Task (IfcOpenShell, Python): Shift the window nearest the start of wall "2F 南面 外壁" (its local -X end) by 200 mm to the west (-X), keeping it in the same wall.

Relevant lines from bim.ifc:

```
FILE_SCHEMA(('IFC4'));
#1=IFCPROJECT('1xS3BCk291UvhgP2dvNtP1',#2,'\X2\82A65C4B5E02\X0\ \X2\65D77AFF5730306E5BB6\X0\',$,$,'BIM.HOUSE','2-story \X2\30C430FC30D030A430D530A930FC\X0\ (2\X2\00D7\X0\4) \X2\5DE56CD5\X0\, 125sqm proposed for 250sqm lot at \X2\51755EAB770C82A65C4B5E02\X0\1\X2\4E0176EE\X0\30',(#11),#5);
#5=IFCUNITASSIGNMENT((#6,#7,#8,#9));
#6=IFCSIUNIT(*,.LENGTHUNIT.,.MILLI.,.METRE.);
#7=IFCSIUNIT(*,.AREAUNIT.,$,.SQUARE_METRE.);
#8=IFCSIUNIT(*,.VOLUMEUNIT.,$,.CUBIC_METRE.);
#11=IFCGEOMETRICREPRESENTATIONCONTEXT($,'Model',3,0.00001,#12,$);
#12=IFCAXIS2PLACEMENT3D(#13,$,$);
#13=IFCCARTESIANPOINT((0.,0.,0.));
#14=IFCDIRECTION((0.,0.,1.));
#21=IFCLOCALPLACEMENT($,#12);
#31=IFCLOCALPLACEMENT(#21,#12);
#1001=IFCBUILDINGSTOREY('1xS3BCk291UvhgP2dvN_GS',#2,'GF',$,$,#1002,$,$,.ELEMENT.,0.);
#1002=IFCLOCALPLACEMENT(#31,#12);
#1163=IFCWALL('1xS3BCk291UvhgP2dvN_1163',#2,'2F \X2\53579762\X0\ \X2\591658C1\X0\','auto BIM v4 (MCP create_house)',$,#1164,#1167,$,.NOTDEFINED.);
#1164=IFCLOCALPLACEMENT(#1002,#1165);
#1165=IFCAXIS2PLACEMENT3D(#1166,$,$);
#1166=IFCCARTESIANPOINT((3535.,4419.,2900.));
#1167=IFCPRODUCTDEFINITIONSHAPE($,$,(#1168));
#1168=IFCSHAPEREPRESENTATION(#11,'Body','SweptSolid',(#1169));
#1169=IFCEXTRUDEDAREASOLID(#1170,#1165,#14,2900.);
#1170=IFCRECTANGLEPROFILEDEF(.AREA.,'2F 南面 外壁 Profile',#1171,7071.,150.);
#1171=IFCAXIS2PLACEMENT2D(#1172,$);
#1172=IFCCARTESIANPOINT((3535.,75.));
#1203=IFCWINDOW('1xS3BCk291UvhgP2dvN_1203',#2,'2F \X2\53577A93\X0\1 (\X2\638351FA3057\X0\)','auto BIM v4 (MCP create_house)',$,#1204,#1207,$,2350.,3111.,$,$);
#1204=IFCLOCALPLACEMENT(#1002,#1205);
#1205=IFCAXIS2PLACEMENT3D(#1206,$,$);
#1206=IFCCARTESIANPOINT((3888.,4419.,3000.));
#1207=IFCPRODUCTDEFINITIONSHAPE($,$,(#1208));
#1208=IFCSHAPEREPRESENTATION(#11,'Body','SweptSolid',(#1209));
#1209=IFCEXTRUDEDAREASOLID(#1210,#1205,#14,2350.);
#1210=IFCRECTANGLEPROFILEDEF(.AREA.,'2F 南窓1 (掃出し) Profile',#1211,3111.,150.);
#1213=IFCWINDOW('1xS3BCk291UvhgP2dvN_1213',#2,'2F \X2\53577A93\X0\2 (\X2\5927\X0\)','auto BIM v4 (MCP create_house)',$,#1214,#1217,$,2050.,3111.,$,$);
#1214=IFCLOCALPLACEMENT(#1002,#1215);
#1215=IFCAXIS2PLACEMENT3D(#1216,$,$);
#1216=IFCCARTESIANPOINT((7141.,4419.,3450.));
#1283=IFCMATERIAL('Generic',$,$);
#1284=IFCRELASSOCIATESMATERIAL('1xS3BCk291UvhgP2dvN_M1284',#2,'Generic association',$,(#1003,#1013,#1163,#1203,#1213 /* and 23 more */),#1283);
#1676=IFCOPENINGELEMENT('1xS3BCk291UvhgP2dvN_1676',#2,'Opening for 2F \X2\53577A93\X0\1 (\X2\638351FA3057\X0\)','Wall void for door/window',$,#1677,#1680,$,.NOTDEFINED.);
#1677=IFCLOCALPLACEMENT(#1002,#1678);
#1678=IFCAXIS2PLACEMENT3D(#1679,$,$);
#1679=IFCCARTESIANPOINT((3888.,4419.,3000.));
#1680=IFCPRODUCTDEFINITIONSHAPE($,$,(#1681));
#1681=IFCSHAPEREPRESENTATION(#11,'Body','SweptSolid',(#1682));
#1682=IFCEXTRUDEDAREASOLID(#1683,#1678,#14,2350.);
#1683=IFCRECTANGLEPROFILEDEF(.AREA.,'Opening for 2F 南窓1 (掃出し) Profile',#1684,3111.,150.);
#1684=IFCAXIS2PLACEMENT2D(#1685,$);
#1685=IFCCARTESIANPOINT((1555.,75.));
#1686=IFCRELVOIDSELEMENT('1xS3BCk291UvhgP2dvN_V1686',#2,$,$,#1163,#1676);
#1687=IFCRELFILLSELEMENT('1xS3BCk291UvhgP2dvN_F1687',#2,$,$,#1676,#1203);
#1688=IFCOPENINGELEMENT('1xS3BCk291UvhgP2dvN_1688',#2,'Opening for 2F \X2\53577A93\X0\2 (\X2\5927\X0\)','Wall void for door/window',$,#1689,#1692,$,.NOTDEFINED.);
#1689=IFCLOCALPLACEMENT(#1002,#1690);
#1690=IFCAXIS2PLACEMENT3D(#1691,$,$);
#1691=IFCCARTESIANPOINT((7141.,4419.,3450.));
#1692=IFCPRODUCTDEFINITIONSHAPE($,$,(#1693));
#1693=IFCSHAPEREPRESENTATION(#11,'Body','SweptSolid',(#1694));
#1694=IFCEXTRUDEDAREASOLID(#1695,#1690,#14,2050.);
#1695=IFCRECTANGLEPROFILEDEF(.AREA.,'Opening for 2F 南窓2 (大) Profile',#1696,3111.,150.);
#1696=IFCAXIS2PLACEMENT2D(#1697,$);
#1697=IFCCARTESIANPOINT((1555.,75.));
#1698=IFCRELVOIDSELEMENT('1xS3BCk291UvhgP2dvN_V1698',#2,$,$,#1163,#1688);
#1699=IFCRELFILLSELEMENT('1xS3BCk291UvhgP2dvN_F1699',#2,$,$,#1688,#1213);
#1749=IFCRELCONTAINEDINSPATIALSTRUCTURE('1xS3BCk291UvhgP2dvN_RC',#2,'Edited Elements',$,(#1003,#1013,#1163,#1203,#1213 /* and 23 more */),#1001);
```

```python
import ifcopenshell
import ifcopenshell.api.geometry
import ifcopenshell.util.placement
import ifcopenshell.util.unit

model = ifcopenshell.open("bim.ifc")
unit_scale = ifcopenshell.util.unit.calculate_unit_scale(model)

window = model.by_guid("1xS3BCk291UvhgP2dvN_1203")
opening = window.FillsVoids[0].RelatingOpeningElement
wall = opening.VoidsElements[0].RelatingBuildingElement

wall_matrix = ifcopenshell.util.placement.get_local_placement(wall.ObjectPlacement)
shift = wall_matrix[:3, 0] * -0.2 / unit_scale
before = ifcopenshell.util.placement.get_local_placement(window.ObjectPlacement)[:3, 3].copy()

# The window is not placed relative to its opening, so move both.
for product in (opening, window):
    matrix = ifcopenshell.util.placement.get_local_placement(product.ObjectPlacement)
    matrix[:3, 3] += shift
    ifcopenshell.api.geometry.edit_object_placement(model, product=product, matrix=matrix, is_si=False)

after = ifcopenshell.util.placement.get_local_placement(window.ObjectPlacement)[:3, 3]
print("window moved by", (after - before).round(3) + 0.0)

model.write("bim_edited.ifc")
```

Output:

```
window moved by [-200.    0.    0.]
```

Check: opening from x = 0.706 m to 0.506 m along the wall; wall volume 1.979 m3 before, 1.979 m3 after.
